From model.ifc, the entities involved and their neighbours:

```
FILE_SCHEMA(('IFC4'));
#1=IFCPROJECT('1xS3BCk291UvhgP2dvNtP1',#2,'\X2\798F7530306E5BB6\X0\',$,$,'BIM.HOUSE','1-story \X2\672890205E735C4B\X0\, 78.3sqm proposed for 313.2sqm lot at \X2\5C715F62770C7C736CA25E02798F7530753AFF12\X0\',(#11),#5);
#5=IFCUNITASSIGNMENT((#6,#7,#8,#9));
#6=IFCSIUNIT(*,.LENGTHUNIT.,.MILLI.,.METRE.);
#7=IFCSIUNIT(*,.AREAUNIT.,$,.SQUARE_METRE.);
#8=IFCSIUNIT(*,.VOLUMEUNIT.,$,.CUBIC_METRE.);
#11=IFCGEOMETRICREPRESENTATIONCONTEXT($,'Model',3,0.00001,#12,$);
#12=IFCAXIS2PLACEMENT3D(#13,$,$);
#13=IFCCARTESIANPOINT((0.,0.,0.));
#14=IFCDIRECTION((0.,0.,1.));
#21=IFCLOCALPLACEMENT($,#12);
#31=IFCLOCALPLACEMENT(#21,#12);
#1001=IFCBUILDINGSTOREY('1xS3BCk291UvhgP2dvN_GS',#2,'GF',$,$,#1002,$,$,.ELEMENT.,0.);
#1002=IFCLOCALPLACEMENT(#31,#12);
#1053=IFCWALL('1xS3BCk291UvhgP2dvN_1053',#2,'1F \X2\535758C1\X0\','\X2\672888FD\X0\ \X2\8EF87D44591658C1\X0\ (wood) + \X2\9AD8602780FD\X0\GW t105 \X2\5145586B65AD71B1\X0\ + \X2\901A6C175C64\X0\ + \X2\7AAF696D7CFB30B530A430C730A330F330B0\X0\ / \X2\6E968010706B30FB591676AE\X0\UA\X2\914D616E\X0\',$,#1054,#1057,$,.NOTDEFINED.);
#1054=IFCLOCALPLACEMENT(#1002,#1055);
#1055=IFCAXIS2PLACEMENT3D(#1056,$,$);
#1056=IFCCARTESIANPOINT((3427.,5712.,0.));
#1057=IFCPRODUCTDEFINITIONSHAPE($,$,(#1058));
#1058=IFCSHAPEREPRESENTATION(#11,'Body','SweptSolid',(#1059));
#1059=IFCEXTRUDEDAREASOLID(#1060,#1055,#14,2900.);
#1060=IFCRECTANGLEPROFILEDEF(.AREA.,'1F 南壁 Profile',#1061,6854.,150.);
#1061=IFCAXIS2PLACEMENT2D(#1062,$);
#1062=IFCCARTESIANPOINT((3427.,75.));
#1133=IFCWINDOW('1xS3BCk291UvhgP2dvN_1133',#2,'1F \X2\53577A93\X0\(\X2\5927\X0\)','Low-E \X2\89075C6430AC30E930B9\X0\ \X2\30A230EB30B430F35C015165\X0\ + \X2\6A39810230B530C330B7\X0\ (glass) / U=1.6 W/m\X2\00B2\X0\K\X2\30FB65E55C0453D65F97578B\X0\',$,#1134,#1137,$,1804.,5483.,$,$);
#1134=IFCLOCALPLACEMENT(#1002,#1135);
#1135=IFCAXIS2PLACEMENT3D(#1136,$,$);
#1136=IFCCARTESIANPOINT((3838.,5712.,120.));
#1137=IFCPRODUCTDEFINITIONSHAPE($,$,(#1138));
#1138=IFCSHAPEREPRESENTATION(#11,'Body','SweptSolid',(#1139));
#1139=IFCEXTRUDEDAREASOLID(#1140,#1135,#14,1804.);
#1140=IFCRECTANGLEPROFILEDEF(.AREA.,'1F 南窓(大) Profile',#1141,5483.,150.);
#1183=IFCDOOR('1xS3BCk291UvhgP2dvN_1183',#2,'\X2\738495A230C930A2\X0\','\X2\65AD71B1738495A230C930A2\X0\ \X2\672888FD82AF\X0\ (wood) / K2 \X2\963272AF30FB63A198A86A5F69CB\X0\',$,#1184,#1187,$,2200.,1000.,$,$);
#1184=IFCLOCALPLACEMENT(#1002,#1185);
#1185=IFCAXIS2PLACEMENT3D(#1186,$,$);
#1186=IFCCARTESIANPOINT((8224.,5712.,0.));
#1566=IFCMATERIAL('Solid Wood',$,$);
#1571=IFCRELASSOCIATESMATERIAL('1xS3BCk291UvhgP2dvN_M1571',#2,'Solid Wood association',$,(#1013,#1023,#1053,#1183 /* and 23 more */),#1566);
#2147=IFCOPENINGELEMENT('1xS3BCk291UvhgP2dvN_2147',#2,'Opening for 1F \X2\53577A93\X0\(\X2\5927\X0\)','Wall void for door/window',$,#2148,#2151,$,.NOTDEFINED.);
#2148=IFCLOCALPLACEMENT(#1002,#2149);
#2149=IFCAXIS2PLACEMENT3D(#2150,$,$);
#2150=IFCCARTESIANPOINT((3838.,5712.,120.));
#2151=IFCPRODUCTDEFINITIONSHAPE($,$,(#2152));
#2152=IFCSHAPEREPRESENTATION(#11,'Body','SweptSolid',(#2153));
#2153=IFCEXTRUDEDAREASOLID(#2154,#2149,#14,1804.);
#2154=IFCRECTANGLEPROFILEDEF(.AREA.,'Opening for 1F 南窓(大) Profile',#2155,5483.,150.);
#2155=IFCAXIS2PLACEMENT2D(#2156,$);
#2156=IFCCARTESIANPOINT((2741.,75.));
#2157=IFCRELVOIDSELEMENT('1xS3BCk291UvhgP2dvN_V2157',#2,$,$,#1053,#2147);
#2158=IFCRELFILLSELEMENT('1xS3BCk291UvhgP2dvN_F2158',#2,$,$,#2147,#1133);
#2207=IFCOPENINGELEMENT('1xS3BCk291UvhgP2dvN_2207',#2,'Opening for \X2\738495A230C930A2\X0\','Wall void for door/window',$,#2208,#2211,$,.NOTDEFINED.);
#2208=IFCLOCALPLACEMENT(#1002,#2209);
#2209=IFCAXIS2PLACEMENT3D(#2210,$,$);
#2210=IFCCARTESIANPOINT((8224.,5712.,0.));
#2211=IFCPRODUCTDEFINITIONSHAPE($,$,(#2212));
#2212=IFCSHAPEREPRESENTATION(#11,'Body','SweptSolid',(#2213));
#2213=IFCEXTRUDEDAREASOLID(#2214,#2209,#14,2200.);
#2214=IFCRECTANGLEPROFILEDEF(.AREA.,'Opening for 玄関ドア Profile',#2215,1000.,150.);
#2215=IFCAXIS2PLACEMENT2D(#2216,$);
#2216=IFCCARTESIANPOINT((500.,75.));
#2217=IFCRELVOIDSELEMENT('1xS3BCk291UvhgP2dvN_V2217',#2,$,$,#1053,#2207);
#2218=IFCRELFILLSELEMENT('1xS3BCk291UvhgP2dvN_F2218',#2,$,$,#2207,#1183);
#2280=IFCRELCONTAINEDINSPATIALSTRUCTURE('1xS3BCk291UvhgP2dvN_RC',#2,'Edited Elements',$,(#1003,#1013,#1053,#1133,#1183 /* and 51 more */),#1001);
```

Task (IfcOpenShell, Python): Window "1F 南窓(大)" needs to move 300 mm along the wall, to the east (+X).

```python
import ifcopenshell
import ifcopenshell.api.geometry
import ifcopenshell.util.placement
import ifcopenshell.util.unit

model = ifcopenshell.open("model.ifc")
unit_scale = ifcopenshell.util.unit.calculate_unit_scale(model)

window = model.by_guid("1xS3BCk291UvhgP2dvN_1133")
opening = window.FillsVoids[0].RelatingOpeningElement
wall = opening.VoidsElements[0].RelatingBuildingElement

wall_matrix = ifcopenshell.util.placement.get_local_placement(wall.ObjectPlacement)
shift = wall_matrix[:3, 0] * 0.3 / unit_scale
before = ifcopenshell.util.placement.get_local_placement(window.ObjectPlacement)[:3, 3].copy()

# The window is not placed relative to its opening, so move both.
for product in (opening, window):
    matrix = ifcopenshell.util.placement.get_local_placement(product.ObjectPlacement)
    matrix[:3, 3] += shift
    ifcopenshell.api.geometry.edit_object_placement(model, product=product, matrix=matrix, is_si=False)

after = ifcopenshell.util.placement.get_local_placement(window.ObjectPlacement)[:3, 3]
print("window moved by", (after - before).round(3) + 0.0)

model.write("model-out.ifc")
```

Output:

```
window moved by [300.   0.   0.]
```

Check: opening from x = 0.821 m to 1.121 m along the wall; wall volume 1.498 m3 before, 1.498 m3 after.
